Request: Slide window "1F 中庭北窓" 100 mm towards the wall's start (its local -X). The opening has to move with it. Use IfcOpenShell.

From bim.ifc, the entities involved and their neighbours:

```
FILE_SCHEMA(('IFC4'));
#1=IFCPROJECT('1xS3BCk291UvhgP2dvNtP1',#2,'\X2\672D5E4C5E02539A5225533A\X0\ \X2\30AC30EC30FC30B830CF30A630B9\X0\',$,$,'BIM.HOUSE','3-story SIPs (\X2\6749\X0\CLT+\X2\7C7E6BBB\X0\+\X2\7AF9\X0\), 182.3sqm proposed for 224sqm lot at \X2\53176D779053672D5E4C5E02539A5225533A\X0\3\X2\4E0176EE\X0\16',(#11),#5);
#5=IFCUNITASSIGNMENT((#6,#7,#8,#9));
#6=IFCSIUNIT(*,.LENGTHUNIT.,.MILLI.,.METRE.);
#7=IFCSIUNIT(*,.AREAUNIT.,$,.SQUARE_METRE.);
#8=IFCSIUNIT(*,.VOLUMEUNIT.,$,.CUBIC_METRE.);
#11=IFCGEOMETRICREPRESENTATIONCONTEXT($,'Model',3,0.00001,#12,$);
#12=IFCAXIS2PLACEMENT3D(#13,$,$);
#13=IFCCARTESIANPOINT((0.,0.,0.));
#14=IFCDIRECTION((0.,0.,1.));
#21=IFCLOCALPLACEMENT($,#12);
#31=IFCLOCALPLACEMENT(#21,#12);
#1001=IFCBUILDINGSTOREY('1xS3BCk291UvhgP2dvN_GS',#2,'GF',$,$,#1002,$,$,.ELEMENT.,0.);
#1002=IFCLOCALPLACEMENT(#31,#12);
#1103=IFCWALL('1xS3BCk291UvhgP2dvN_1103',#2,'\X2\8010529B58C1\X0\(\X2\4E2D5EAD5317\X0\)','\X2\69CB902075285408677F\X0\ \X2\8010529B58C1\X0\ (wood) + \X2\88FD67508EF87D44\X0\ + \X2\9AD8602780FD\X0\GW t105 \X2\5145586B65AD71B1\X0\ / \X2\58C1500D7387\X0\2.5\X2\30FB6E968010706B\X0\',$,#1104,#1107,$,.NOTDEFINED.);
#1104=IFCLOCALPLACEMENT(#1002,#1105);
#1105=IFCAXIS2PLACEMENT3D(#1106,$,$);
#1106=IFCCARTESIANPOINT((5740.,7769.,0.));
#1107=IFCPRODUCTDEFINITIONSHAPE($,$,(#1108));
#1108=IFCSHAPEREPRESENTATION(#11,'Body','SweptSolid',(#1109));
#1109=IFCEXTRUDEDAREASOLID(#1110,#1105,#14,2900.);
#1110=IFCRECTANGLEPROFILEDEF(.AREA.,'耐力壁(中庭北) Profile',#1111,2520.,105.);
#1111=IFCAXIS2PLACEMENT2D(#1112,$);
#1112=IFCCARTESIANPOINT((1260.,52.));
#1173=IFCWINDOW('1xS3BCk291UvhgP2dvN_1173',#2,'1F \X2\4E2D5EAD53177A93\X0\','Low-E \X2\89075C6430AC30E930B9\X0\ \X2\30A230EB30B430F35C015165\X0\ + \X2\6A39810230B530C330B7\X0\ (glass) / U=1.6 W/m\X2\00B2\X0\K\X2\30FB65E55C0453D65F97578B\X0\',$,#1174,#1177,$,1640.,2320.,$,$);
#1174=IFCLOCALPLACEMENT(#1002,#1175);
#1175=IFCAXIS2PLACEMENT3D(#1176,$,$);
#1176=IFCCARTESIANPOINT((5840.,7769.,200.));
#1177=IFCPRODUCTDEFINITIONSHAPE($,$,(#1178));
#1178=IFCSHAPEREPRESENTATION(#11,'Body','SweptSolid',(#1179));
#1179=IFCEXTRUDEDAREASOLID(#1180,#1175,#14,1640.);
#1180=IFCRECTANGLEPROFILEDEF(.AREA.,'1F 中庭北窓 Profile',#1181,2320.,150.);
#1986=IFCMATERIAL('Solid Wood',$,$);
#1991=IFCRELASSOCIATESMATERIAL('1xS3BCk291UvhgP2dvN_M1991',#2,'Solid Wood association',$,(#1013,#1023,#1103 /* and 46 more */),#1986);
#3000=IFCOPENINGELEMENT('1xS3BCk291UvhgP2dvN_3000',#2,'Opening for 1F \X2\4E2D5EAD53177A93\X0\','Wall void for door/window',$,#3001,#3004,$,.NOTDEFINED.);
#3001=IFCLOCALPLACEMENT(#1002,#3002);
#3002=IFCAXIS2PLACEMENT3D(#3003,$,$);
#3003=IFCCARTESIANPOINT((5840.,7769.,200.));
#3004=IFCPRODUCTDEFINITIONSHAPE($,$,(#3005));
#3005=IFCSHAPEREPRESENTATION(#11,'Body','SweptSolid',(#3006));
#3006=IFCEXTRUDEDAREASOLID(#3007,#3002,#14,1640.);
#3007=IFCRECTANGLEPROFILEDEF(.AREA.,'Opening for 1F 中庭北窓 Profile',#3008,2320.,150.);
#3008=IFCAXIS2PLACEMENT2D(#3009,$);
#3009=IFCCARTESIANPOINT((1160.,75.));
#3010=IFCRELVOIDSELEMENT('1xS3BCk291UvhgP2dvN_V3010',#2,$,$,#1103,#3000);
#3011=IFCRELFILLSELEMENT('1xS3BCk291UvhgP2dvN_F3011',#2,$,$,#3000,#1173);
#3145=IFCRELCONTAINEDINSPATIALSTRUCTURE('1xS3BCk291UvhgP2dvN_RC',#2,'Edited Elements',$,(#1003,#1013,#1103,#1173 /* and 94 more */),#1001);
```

```python
import ifcopenshell
import ifcopenshell.api.geometry
import ifcopenshell.util.placement
import ifcopenshell.util.unit

model = ifcopenshell.open("bim.ifc")
unit_scale = ifcopenshell.util.unit.calculate_unit_scale(model)

window = model.by_guid("1xS3BCk291UvhgP2dvN_1173")
opening = window.FillsVoids[0].RelatingOpeningElement
wall = opening.VoidsElements[0].RelatingBuildingElement

wall_matrix = ifcopenshell.util.placement.get_local_placement(wall.ObjectPlacement)
shift = wall_matrix[:3, 0] * -0.1 / unit_scale
before = ifcopenshell.util.placement.get_local_placement(window.ObjectPlacement)[:3, 3].copy()

# The window is not placed relative to its opening, so move both.
for product in (opening, window):
    matrix = ifcopenshell.util.placement.get_local_placement(product.ObjectPlacement)
    matrix[:3, 3] += shift
    ifcopenshell.api.geometry.edit_object_placement(model, product=product, matrix=matrix, is_si=False)

after = ifcopenshell.util.placement.get_local_placement(window.ObjectPlacement)[:3, 3]
print("window moved by", (after - before).round(3) + 0.0)

model.write("bim_updated.ifc")
```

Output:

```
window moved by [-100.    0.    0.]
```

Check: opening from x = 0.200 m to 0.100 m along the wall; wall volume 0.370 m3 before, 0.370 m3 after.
